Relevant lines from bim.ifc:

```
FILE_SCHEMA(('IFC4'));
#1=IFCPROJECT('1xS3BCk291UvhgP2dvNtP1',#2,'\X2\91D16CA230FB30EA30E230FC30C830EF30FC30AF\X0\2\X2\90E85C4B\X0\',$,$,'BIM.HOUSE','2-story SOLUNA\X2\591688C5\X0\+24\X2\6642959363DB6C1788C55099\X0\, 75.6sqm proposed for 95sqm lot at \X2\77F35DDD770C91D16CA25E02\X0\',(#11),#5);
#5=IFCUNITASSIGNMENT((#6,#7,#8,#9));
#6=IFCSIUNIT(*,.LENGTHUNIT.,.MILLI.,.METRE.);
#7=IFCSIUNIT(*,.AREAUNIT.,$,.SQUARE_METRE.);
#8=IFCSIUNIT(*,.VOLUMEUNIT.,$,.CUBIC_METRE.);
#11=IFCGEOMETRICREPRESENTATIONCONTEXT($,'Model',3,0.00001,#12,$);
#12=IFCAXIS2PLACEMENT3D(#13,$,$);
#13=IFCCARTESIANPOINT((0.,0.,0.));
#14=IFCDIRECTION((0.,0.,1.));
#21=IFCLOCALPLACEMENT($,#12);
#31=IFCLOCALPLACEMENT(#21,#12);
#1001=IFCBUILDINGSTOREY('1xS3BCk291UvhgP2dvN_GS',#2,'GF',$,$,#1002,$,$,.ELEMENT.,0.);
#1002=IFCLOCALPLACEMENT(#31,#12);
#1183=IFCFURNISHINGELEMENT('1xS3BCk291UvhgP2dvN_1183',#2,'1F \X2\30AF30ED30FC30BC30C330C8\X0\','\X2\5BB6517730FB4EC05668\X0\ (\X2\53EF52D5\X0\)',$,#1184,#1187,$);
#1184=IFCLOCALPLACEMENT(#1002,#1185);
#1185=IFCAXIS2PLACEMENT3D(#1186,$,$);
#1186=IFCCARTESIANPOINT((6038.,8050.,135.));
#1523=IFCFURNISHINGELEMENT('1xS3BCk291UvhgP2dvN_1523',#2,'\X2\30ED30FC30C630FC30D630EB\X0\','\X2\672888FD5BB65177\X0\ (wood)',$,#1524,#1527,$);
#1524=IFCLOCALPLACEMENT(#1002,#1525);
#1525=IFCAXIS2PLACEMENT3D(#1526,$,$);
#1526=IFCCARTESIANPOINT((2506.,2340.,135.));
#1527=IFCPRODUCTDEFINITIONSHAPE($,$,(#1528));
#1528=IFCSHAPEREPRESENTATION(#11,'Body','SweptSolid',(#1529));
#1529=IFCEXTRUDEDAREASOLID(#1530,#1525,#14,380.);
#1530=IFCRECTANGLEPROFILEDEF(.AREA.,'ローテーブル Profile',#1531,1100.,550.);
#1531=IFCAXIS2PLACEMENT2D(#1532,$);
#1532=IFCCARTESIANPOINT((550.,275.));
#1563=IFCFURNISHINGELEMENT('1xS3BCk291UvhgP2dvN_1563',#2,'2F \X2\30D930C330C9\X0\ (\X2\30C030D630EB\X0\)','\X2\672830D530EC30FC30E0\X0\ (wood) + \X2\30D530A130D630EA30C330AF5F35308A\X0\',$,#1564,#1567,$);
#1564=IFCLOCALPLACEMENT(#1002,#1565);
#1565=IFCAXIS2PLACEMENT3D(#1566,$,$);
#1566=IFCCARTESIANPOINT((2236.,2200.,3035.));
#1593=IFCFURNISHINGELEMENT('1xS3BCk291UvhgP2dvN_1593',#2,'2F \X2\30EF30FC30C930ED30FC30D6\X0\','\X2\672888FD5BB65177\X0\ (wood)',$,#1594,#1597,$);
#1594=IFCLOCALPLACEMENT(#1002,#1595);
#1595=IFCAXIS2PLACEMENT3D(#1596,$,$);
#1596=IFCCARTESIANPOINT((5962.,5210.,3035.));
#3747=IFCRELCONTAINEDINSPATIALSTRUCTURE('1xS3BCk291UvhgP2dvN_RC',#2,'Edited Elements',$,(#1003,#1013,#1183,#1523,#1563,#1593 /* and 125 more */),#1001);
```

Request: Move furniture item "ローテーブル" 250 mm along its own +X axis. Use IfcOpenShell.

```python
import ifcopenshell
import ifcopenshell.api.geometry
import ifcopenshell.util.placement
import ifcopenshell.util.unit

model = ifcopenshell.open("bim.ifc")
unit_scale = ifcopenshell.util.unit.calculate_unit_scale(model)

item = model.by_guid("1xS3BCk291UvhgP2dvN_1523")
matrix = ifcopenshell.util.placement.get_local_placement(item.ObjectPlacement)
matrix[:3, 3] += matrix[:3, 0] * 0.25 / unit_scale
ifcopenshell.api.geometry.edit_object_placement(model, product=item, matrix=matrix, is_si=False)

print(ifcopenshell.util.placement.get_local_placement(item.ObjectPlacement).round(3) + 0.0)

model.write("bim_v2.ifc")
```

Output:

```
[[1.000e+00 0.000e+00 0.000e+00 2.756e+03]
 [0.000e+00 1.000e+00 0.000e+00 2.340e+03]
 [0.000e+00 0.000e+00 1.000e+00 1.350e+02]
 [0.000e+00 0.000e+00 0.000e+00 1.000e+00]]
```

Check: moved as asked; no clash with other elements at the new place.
